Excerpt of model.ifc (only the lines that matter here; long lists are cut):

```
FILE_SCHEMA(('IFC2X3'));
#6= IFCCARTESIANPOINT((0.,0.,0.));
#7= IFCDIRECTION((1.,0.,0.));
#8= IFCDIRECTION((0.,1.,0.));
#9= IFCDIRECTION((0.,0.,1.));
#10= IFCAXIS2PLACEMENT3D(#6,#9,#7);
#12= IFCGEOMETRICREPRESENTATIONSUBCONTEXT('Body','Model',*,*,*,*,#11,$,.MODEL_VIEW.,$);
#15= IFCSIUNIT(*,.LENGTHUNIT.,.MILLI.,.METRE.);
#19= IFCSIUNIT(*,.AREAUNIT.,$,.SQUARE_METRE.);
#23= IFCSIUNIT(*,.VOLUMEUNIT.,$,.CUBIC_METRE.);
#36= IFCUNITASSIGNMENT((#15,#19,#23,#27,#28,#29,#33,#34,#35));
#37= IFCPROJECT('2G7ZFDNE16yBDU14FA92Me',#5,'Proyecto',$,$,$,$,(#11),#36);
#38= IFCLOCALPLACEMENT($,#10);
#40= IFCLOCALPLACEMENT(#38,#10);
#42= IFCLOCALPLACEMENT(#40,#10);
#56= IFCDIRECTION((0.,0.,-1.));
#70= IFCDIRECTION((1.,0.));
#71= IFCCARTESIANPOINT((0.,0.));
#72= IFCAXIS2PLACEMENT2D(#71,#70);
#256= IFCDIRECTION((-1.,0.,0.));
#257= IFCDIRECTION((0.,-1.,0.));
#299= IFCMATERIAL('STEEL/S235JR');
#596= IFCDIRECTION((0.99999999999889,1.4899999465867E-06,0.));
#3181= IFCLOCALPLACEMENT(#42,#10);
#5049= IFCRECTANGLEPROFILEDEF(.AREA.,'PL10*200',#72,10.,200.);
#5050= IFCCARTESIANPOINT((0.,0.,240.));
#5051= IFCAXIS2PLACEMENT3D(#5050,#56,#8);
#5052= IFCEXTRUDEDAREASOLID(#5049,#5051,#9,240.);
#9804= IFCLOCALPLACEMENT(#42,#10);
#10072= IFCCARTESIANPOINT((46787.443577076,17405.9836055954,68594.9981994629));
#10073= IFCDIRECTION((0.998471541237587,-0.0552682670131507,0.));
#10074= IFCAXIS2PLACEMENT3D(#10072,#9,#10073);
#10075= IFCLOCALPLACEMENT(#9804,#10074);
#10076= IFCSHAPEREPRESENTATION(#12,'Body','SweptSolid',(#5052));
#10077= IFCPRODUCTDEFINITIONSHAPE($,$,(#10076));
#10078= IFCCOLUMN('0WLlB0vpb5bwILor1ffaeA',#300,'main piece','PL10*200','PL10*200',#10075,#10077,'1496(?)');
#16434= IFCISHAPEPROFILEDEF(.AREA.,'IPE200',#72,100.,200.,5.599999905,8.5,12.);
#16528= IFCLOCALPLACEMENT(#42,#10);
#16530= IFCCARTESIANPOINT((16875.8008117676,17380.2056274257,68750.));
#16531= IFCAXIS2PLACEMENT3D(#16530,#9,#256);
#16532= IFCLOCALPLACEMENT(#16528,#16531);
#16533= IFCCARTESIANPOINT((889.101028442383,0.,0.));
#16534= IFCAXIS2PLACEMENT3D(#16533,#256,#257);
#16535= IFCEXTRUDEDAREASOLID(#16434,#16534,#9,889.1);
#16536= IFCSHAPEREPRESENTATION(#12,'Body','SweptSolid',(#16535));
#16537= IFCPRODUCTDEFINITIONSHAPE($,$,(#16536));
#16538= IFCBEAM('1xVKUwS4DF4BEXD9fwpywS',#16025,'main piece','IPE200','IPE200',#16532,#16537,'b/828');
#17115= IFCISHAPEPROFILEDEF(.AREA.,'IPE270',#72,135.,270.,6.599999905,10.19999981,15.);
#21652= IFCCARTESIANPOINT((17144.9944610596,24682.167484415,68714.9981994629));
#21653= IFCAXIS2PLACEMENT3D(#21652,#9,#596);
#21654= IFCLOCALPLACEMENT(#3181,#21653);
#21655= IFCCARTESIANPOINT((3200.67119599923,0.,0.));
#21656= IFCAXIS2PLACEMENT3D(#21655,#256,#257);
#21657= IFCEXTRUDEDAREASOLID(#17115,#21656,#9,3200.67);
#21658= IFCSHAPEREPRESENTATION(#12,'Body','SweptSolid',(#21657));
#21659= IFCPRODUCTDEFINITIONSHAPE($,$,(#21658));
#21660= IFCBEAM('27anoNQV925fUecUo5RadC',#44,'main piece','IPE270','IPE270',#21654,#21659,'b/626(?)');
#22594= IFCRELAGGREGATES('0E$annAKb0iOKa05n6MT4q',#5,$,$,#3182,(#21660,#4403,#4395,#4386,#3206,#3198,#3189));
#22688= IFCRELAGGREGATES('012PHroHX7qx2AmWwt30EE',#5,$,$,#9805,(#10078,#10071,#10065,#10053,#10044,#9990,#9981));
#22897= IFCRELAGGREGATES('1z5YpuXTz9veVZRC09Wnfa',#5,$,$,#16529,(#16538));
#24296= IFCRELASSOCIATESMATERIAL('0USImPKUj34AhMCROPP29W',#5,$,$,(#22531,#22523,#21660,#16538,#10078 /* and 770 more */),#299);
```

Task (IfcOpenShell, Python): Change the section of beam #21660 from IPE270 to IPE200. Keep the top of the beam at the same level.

```python
import ifcopenshell
import ifcopenshell.util.element
import ifcopenshell.util.representation

model = ifcopenshell.open("model.ifc")

member = model.by_guid("27anoNQV925fUecUo5RadC")
source = next(p for p in model.by_type("IfcIShapeProfileDef") if p.ProfileName == "IPE200")

body = ifcopenshell.util.representation.get_representation(member, "Model", "Body")
solid = body.Items[0]
old_profile = solid.SweptArea

# Copy the section's sizes but keep this member's own profile position.
profile = ifcopenshell.util.element.copy(model, source)
# Profiles are centred, so shift by half the change in depth to hold the top.
shift = (old_profile.OverallDepth - profile.OverallDepth) / 2
x, y = old_profile.Position.Location.Coordinates
up = (0.0, 1.0)  # upwards, in the solid's own plane
location = model.createIfcCartesianPoint((x + up[0] * shift, y + up[1] * shift))
profile.Position = model.createIfcAxis2Placement2D(location, old_profile.Position.RefDirection)
solid.SweptArea = profile
if not model.get_total_inverses(old_profile):
    ifcopenshell.util.element.remove_deep2(model, old_profile)
member.Description = member.Description.replace("IPE270", "IPE200")
member.ObjectType = member.ObjectType.replace("IPE270", "IPE200")

print(solid.SweptArea)

model.write("model-out.ifc")
```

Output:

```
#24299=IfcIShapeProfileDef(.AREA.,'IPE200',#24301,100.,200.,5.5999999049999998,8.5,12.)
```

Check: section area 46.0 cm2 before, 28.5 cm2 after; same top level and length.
